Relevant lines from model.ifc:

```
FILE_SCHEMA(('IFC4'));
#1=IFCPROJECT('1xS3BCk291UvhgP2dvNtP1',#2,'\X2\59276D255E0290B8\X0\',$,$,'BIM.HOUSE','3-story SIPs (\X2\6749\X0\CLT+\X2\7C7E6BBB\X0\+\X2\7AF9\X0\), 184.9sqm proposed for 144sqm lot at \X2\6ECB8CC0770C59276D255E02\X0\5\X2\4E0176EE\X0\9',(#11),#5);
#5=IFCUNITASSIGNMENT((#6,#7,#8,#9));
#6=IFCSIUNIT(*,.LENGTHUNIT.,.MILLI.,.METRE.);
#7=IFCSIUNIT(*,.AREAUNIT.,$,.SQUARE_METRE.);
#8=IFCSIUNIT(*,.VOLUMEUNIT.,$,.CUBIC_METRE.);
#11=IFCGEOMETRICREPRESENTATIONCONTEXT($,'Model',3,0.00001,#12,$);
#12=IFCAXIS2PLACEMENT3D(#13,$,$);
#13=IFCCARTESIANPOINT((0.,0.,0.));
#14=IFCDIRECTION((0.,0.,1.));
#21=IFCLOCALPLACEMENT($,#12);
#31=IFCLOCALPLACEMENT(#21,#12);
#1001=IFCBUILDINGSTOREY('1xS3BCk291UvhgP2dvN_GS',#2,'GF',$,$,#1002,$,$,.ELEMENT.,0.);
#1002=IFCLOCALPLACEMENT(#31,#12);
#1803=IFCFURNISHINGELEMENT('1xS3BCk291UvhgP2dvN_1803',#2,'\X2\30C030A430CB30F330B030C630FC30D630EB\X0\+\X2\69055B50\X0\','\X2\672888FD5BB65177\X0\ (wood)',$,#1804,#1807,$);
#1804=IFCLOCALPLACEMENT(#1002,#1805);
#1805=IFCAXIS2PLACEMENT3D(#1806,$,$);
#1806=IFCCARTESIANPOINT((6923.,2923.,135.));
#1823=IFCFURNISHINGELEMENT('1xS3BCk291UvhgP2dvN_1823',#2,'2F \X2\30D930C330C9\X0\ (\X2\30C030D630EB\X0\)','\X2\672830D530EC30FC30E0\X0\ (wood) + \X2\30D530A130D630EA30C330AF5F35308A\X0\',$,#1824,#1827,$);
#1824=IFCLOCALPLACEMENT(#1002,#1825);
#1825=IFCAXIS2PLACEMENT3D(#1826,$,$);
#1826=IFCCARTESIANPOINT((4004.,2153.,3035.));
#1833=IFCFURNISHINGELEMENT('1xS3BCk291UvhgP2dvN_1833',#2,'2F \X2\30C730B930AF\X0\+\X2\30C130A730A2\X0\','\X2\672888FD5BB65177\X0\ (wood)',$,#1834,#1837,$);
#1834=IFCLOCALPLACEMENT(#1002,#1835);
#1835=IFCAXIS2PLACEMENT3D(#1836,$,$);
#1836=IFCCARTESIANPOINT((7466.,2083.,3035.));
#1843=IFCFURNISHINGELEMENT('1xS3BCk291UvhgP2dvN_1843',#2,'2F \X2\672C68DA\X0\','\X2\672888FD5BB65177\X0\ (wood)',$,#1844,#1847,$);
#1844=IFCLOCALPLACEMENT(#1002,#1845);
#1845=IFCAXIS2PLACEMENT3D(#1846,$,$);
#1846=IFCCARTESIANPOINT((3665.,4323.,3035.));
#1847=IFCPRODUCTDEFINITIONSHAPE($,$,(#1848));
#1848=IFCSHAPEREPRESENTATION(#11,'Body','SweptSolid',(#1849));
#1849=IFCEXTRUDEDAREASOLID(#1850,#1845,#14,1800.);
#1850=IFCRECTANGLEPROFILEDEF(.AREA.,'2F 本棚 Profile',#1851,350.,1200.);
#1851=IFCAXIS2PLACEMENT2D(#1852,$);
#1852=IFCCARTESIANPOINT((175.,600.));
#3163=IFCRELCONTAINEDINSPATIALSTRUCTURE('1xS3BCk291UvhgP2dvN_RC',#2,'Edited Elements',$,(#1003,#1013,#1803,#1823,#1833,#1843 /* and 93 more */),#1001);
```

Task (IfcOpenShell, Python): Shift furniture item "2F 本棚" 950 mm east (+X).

```python
import ifcopenshell
import ifcopenshell.api.geometry
import ifcopenshell.util.placement
import ifcopenshell.util.unit

model = ifcopenshell.open("model.ifc")
unit_scale = ifcopenshell.util.unit.calculate_unit_scale(model)

item = model.by_guid("1xS3BCk291UvhgP2dvN_1843")
matrix = ifcopenshell.util.placement.get_local_placement(item.ObjectPlacement)
matrix[0, 3] += 0.95 / unit_scale
ifcopenshell.api.geometry.edit_object_placement(model, product=item, matrix=matrix, is_si=False)

print(ifcopenshell.util.placement.get_local_placement(item.ObjectPlacement).round(3) + 0.0)

model.write("model_edited.ifc")
```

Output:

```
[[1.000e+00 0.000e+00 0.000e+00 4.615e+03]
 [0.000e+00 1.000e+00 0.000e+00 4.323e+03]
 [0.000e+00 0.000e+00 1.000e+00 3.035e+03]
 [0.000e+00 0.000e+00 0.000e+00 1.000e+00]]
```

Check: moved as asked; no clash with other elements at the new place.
